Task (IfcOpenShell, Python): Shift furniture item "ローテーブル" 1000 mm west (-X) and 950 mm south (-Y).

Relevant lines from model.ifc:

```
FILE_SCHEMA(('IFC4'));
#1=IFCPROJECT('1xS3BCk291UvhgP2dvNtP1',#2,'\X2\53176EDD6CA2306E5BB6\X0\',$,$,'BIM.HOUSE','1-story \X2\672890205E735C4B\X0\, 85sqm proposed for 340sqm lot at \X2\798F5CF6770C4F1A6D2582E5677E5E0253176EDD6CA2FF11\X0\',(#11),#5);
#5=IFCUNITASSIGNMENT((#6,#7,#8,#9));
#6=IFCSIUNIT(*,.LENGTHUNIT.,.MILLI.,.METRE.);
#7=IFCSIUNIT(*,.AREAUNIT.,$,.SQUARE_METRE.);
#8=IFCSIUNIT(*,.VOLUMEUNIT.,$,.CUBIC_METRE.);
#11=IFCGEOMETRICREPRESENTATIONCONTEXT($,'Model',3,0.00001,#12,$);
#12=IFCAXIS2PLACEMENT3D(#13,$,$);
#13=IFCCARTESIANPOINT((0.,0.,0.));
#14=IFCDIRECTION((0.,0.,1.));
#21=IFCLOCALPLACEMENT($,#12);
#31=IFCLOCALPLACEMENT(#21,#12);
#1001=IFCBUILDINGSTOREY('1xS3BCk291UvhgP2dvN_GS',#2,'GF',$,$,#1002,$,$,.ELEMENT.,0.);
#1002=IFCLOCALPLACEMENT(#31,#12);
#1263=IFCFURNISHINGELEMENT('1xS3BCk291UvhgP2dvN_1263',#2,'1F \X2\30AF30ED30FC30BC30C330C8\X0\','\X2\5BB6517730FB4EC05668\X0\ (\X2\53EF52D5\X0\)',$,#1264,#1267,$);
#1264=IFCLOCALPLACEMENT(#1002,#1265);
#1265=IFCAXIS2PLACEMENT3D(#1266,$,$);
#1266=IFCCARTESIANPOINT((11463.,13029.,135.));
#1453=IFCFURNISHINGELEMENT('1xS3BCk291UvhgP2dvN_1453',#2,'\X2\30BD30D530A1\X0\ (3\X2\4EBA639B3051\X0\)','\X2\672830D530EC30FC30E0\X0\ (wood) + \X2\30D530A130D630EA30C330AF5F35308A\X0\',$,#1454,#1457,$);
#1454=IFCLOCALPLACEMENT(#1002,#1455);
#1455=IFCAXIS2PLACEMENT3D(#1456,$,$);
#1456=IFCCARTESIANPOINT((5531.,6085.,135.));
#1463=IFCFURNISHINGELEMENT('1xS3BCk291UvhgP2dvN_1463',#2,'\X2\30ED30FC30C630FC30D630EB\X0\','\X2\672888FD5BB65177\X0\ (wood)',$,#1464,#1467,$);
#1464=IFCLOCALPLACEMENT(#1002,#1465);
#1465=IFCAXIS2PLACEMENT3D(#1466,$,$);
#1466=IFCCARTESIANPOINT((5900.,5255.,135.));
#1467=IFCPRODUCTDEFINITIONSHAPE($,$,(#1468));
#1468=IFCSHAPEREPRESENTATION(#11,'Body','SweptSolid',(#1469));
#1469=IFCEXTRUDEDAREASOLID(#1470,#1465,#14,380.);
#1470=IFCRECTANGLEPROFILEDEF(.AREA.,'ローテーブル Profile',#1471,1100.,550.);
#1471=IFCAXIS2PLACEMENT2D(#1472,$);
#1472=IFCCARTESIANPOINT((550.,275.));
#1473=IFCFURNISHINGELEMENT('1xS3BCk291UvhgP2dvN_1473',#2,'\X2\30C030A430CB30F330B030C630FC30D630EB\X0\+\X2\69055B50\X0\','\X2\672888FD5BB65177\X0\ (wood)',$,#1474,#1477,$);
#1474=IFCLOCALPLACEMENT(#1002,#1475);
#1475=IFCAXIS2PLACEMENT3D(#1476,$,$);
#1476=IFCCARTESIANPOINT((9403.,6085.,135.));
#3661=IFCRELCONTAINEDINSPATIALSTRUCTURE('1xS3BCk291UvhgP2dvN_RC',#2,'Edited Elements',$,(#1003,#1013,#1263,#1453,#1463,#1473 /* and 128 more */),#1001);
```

```python
import ifcopenshell
import ifcopenshell.api.geometry
import ifcopenshell.util.placement
import ifcopenshell.util.unit

model = ifcopenshell.open("model.ifc")
unit_scale = ifcopenshell.util.unit.calculate_unit_scale(model)

item = model.by_guid("1xS3BCk291UvhgP2dvN_1463")
matrix = ifcopenshell.util.placement.get_local_placement(item.ObjectPlacement)
matrix[0, 3] -= 1 / unit_scale
matrix[1, 3] -= 0.95 / unit_scale
ifcopenshell.api.geometry.edit_object_placement(model, product=item, matrix=matrix, is_si=False)

print(ifcopenshell.util.placement.get_local_placement(item.ObjectPlacement).round(3) + 0.0)

model.write("model_v2.ifc")
```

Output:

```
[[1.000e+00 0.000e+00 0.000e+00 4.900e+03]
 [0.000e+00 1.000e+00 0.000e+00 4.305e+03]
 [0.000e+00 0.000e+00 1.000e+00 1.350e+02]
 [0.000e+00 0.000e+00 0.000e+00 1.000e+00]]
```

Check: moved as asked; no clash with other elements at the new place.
